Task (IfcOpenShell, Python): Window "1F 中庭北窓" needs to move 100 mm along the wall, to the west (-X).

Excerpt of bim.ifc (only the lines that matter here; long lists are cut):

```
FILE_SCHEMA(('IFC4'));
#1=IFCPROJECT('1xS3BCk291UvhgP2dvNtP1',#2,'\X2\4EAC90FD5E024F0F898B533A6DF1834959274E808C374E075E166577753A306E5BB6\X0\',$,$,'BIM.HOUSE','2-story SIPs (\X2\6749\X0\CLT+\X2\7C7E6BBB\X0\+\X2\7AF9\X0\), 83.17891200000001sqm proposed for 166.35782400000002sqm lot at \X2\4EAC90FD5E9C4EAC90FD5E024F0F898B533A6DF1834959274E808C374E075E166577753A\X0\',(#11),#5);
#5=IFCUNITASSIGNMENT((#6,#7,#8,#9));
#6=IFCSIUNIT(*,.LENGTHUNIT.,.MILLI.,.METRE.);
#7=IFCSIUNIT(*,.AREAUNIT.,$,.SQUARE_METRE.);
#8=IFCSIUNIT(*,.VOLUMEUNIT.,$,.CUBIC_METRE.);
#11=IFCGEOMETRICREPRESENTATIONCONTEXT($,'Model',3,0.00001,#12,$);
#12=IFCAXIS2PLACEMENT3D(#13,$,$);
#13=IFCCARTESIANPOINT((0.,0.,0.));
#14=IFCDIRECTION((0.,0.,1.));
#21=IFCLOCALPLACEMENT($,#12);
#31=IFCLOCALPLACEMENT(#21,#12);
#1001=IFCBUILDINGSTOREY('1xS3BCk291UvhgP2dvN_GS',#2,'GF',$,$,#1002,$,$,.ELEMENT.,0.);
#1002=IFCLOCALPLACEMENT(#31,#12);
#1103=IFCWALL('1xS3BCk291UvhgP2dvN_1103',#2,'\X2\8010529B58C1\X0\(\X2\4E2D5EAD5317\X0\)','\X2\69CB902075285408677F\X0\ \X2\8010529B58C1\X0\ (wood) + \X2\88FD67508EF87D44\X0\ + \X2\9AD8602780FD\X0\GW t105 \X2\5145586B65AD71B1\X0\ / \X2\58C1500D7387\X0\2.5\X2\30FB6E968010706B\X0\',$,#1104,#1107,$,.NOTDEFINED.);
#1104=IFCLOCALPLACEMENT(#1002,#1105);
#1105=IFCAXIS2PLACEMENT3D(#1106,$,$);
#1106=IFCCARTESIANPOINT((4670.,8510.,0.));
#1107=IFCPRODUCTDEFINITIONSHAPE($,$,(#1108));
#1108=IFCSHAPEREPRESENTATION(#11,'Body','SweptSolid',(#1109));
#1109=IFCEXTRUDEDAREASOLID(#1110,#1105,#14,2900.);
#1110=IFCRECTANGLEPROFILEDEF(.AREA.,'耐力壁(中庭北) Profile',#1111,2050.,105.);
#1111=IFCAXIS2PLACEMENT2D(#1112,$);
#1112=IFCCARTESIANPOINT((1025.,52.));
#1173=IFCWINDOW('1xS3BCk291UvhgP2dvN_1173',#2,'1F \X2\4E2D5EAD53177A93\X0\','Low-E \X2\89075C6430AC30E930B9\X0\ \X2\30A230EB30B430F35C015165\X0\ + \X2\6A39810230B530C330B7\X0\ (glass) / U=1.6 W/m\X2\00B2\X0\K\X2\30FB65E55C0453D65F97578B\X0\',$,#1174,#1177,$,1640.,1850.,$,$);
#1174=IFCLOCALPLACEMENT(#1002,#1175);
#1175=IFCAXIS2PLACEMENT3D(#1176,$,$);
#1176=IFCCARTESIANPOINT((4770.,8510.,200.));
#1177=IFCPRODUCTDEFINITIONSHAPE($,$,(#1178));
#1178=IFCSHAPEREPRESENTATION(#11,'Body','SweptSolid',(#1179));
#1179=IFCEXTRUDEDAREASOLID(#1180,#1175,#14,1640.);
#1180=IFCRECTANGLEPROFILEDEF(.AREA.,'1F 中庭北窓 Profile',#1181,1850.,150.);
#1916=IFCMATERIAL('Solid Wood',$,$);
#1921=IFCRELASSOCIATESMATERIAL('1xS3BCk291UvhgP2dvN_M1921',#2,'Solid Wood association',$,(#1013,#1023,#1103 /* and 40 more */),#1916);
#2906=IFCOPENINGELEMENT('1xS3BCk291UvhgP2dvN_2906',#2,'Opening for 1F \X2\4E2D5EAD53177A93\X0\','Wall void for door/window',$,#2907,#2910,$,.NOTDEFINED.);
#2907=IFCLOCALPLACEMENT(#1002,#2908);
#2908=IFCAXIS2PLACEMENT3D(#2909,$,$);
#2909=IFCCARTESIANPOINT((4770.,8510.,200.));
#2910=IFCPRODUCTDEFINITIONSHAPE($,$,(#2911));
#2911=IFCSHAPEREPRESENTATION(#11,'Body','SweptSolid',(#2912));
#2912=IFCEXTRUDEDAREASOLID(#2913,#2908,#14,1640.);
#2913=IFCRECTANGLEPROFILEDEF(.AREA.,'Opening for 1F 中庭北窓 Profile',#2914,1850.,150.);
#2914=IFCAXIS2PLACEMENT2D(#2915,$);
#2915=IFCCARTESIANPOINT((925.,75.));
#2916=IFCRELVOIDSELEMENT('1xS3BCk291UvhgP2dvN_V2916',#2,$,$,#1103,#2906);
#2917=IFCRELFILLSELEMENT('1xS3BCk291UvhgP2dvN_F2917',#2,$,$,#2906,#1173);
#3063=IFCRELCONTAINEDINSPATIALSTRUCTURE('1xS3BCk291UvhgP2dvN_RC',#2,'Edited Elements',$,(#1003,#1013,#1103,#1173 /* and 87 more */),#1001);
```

```python
import ifcopenshell
import ifcopenshell.api.geometry
import ifcopenshell.util.placement
import ifcopenshell.util.unit

model = ifcopenshell.open("bim.ifc")
unit_scale = ifcopenshell.util.unit.calculate_unit_scale(model)

window = model.by_id(1173)
opening = window.FillsVoids[0].RelatingOpeningElement
wall = opening.VoidsElements[0].RelatingBuildingElement

wall_matrix = ifcopenshell.util.placement.get_local_placement(wall.ObjectPlacement)
shift = wall_matrix[:3, 0] * -0.1 / unit_scale
before = ifcopenshell.util.placement.get_local_placement(window.ObjectPlacement)[:3, 3].copy()

# The window is not placed relative to its opening, so move both.
for product in (opening, window):
    matrix = ifcopenshell.util.placement.get_local_placement(product.ObjectPlacement)
    matrix[:3, 3] += shift
    ifcopenshell.api.geometry.edit_object_placement(model, product=product, matrix=matrix, is_si=False)

after = ifcopenshell.util.placement.get_local_placement(window.ObjectPlacement)[:3, 3]
print("window moved by", (after - before).round(3) + 0.0)

model.write("bim-out.ifc")
```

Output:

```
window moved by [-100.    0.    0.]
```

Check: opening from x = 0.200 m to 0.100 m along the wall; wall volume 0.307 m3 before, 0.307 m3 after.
